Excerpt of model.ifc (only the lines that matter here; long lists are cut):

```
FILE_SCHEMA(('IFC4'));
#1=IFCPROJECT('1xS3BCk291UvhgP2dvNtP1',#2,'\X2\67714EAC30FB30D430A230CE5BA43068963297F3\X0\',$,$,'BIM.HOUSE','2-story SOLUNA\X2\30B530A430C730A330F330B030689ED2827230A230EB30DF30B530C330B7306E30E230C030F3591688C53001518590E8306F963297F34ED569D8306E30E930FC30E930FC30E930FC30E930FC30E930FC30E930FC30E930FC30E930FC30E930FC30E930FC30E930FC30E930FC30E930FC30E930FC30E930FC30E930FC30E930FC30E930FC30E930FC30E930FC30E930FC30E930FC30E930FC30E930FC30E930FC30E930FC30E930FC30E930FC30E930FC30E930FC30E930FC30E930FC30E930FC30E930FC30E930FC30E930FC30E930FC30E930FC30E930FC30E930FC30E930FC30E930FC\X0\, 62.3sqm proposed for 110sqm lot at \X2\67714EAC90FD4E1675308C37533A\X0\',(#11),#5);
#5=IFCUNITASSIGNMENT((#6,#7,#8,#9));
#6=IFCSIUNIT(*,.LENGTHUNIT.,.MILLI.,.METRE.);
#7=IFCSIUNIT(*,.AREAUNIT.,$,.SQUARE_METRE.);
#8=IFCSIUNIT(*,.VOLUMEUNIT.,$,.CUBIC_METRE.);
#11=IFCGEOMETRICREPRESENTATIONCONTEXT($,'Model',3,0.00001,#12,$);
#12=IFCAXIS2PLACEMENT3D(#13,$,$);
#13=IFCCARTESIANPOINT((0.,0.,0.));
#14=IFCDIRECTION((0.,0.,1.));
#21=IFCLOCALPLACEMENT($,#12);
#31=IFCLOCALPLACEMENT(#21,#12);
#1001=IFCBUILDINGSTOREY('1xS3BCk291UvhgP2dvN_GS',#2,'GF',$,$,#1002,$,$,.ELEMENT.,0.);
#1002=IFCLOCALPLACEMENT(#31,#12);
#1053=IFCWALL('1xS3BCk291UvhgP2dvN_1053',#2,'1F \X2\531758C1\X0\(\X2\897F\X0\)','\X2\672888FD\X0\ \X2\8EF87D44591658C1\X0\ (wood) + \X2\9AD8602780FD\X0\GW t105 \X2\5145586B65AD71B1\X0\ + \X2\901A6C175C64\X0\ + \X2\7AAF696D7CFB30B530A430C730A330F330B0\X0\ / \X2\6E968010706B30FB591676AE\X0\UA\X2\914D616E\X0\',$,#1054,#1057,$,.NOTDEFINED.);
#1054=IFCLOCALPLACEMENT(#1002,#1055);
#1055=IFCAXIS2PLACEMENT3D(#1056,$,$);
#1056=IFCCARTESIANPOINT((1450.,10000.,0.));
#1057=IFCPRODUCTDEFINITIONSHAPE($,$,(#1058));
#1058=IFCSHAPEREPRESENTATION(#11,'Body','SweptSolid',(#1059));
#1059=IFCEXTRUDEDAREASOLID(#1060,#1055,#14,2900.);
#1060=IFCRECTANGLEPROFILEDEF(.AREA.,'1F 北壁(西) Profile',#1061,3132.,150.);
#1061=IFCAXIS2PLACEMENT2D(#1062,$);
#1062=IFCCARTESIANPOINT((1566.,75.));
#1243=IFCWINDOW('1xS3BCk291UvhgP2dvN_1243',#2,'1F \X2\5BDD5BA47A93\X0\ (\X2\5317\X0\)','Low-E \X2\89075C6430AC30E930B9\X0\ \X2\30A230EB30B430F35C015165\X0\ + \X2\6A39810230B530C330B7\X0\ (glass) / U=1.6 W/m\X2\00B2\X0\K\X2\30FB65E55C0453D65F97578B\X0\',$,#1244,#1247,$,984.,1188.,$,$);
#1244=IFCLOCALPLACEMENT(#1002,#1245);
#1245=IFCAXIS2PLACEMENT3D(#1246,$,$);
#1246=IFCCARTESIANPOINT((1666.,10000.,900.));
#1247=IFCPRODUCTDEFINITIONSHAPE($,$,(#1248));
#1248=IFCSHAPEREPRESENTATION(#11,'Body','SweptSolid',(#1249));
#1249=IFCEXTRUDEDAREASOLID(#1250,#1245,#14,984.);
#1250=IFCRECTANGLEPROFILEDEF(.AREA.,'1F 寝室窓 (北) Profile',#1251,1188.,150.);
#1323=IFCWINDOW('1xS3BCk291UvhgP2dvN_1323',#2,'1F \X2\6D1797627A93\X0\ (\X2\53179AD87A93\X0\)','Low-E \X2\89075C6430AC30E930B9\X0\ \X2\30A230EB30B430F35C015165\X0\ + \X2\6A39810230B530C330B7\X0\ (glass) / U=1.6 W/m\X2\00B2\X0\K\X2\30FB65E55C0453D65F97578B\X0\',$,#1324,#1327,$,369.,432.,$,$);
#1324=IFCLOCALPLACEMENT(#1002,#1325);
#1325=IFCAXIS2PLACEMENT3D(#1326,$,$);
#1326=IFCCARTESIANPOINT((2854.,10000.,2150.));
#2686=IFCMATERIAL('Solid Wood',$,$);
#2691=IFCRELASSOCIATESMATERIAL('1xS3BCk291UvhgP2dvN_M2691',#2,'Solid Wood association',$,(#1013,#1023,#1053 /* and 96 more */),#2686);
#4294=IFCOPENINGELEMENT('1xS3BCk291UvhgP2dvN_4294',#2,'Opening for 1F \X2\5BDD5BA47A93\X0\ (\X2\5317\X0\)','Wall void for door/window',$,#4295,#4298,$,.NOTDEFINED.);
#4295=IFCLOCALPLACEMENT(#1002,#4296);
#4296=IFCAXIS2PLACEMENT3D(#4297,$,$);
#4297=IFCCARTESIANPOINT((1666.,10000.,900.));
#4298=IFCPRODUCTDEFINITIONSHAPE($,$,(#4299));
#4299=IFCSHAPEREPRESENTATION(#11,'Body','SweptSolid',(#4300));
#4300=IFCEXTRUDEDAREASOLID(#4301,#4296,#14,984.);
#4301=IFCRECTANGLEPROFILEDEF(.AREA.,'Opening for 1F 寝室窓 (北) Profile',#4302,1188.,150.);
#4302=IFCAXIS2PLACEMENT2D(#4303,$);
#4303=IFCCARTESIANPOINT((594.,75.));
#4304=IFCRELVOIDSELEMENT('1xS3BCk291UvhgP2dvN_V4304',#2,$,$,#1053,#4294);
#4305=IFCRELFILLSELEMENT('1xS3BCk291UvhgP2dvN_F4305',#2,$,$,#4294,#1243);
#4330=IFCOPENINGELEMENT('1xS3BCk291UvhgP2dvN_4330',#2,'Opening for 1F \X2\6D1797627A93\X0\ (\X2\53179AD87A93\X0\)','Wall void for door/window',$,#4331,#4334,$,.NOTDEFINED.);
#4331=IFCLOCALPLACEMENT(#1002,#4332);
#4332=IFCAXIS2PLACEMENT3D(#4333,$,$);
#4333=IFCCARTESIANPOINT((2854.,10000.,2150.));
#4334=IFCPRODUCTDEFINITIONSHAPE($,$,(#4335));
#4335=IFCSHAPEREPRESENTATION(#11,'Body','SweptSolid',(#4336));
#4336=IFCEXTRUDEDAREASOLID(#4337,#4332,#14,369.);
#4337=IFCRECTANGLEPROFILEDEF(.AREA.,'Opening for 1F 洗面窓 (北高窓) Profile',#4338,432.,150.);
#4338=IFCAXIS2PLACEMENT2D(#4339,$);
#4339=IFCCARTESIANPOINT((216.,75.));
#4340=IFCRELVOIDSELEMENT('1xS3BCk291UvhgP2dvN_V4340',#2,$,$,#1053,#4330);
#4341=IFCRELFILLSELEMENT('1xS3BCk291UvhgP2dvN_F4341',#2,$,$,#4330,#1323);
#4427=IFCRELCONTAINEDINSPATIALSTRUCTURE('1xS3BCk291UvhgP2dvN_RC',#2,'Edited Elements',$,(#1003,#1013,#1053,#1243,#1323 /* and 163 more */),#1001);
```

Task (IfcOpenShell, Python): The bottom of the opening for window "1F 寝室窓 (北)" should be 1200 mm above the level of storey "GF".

```python
import numpy as np
import ifcopenshell
import ifcopenshell.api.geometry
import ifcopenshell.geom
import ifcopenshell.util.element
import ifcopenshell.util.placement
import ifcopenshell.util.shape
import ifcopenshell.util.unit

model = ifcopenshell.open("model.ifc")
unit_scale = ifcopenshell.util.unit.calculate_unit_scale(model)

window = model.by_guid("1xS3BCk291UvhgP2dvN_1243")
opening = window.FillsVoids[0].RelatingOpeningElement
storey = ifcopenshell.util.element.get_container(window, ifc_class="IfcBuildingStorey")
level = ifcopenshell.util.placement.get_local_placement(storey.ObjectPlacement)[2, 3]

# The opening's origin need not be at the sill, so measure its lowest point.
shape = ifcopenshell.geom.create_shape(ifcopenshell.geom.settings(), opening)
bottom = ifcopenshell.util.shape.get_shape_bottom_elevation(shape, shape.geometry) / unit_scale
dz = level + 1.2 / unit_scale - bottom

shift = np.array([0.0, 0.0, dz])
# The window is not placed relative to its opening, so move both.
for product in (opening, window):
    matrix = ifcopenshell.util.placement.get_local_placement(product.ObjectPlacement)
    matrix[:3, 3] += shift
    ifcopenshell.api.geometry.edit_object_placement(model, product=product, matrix=matrix, is_si=False)

print(f"moved by {dz * unit_scale:+.3f} m")

model.write("model_rev.ifc")
```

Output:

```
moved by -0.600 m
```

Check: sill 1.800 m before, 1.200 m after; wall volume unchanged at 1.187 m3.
